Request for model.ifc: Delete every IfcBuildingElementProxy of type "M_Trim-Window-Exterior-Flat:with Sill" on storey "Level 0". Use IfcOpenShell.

First a look at what the model holds.

```python
import ifcopenshell
import ifcopenshell.util.element

model = ifcopenshell.open("model.ifc")
print(model.schema)
storey = next(s for s in model.by_type("IfcBuildingStorey") if s.Name == "Level 0")
proxies = [e for e in ifcopenshell.util.element.get_decomposition(storey) if e.is_a("IfcBuildingElementProxy")]
seen = {}
for e in proxies:
    element_type = ifcopenshell.util.element.get_type(e)
    name = element_type.Name if element_type not in (None, e) else None
    seen[name] = seen.get(name, 0) + 1
for name, count in sorted(seen.items(), key=str):
    print(count, "x", name)
```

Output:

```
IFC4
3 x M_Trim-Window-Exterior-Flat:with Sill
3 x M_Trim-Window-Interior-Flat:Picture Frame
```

```python
import ifcopenshell
import ifcopenshell.api.root
import ifcopenshell.util.element

model = ifcopenshell.open("model.ifc")

storey = next(s for s in model.by_type("IfcBuildingStorey") if s.Name == "Level 0")
proxies = [e for e in ifcopenshell.util.element.get_decomposition(storey) if e.is_a("IfcBuildingElementProxy")]
targets = [e for e in proxies if (t := ifcopenshell.util.element.get_type(e)) not in (None, e) and t.Name == "M_Trim-Window-Exterior-Flat:with Sill"]

for e in targets:
    ifcopenshell.api.root.remove_product(model, product=e)
print(len(targets), "removed")

model.write("model-out.ifc")
```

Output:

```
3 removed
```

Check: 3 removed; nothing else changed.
